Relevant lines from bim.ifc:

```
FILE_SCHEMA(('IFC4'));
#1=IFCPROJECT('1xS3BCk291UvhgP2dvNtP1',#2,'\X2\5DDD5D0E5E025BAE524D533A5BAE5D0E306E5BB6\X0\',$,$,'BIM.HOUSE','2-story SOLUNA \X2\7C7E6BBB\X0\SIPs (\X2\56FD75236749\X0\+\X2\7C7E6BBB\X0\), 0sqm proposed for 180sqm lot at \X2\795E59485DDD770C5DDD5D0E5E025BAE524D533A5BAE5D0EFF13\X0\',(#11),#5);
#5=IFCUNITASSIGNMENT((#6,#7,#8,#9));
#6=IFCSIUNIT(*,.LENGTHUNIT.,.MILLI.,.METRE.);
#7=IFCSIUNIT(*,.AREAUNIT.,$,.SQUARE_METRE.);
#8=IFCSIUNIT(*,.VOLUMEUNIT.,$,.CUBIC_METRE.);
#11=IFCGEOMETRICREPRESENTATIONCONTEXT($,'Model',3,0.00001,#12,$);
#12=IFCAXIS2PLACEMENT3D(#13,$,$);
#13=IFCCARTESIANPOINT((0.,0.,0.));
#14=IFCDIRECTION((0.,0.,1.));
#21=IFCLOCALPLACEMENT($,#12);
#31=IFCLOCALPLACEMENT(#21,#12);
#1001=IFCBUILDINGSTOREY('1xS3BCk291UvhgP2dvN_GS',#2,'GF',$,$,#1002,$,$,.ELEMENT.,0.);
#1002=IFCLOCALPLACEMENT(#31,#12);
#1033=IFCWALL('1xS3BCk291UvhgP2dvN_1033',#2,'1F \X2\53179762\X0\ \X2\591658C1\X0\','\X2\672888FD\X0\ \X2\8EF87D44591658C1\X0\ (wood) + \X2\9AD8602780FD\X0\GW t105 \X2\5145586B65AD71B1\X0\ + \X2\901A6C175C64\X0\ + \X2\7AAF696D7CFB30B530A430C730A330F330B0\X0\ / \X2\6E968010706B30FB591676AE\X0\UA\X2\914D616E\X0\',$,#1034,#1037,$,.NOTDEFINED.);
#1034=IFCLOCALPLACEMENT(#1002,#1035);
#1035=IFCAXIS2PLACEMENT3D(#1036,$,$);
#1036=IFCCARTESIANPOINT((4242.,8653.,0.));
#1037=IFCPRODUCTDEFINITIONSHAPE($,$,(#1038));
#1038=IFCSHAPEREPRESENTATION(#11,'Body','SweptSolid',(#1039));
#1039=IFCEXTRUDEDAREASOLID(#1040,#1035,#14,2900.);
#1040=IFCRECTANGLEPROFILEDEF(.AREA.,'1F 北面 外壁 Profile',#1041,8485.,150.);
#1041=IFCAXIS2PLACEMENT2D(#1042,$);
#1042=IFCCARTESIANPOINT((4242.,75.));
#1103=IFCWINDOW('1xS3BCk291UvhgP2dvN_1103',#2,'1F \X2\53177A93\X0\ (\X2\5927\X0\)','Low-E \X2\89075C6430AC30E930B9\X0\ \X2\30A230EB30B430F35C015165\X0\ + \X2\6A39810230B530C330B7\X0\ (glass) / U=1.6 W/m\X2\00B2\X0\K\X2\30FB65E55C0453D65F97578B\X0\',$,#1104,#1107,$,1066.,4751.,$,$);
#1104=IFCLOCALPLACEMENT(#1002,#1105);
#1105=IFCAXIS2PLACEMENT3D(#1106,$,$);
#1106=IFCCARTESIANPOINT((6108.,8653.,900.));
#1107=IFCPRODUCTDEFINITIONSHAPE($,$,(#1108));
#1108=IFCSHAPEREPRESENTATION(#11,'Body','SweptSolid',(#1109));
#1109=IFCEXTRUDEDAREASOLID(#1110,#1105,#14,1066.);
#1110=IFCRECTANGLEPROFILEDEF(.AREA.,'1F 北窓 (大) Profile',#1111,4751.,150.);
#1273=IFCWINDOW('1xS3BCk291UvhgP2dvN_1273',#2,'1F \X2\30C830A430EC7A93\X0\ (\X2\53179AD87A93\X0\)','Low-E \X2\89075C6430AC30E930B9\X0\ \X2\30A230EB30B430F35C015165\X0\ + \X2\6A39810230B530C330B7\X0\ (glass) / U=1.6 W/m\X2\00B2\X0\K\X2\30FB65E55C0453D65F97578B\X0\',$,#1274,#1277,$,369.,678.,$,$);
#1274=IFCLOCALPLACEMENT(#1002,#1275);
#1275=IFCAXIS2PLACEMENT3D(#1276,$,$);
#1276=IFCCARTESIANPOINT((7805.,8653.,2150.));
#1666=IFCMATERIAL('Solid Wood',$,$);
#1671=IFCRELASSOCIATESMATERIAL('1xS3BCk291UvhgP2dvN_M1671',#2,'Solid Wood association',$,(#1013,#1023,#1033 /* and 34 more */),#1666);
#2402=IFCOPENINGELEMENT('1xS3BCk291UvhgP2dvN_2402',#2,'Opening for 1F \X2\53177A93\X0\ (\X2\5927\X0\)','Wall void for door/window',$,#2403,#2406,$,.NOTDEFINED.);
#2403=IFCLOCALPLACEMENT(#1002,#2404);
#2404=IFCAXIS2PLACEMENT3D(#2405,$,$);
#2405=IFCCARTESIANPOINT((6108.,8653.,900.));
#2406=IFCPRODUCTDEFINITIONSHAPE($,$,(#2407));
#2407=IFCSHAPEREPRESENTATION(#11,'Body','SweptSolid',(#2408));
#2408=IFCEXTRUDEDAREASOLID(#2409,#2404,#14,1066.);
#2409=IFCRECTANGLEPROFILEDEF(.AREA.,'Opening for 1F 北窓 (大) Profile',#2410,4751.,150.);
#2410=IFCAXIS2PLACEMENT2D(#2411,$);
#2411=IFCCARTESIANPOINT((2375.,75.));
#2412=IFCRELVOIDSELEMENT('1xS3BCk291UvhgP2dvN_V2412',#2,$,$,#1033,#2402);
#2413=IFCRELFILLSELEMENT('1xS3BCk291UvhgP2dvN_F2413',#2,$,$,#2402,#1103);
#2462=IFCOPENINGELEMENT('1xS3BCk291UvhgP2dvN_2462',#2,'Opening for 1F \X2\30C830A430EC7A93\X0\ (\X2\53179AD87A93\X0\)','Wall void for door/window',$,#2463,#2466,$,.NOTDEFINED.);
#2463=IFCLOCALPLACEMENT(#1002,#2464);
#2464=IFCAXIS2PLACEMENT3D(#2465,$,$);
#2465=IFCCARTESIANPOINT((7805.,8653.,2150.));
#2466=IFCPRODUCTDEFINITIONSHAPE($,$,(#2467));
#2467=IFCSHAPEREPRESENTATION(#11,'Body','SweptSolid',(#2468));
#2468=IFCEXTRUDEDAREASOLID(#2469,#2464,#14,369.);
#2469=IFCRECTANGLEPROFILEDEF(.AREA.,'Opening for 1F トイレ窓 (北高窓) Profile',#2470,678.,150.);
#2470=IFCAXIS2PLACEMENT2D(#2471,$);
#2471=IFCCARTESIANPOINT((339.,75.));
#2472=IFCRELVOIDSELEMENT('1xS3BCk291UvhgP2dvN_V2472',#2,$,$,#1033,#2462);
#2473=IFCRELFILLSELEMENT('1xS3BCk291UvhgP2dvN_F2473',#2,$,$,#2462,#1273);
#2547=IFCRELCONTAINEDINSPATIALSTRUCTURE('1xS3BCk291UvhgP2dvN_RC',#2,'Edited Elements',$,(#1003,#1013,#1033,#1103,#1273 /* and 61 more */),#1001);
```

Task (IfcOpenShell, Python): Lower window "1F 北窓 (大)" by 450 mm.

```python
import numpy as np
import ifcopenshell
import ifcopenshell.api.geometry
import ifcopenshell.util.placement
import ifcopenshell.util.unit

model = ifcopenshell.open("bim.ifc")
unit_scale = ifcopenshell.util.unit.calculate_unit_scale(model)

window = model.by_guid("1xS3BCk291UvhgP2dvN_1103")
opening = window.FillsVoids[0].RelatingOpeningElement
dz = -0.45 / unit_scale

shift = np.array([0.0, 0.0, dz])
# The window is not placed relative to its opening, so move both.
for product in (opening, window):
    matrix = ifcopenshell.util.placement.get_local_placement(product.ObjectPlacement)
    matrix[:3, 3] += shift
    ifcopenshell.api.geometry.edit_object_placement(model, product=product, matrix=matrix, is_si=False)

print(f"moved by {dz * unit_scale:+.3f} m")

model.write("bim_edited.ifc")
```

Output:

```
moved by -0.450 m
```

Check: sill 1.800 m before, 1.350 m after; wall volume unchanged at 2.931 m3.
